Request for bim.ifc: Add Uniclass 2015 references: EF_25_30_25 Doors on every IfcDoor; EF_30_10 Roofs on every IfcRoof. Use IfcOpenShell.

First a look at what the model holds.

```python
import ifcopenshell

model = ifcopenshell.open("bim.ifc")
print(model.schema)
print("classifications:", [c.Name for c in model.by_type("IfcClassification")])
for ifc_class in ("IfcDoor", "IfcRoof", "IfcStair", "IfcWall", "IfcWindow"):
    print(ifc_class, len(model.by_type(ifc_class)))
```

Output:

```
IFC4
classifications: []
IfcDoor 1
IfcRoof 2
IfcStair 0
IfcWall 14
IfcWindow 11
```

```python
import ifcopenshell
import ifcopenshell.api.classification

model = ifcopenshell.open("bim.ifc")

system = ifcopenshell.api.classification.add_classification(model, classification="Uniclass 2015")

codes = {
    "IfcDoor": ("EF_25_30_25", "Doors"),
    "IfcRoof": ("EF_30_10", "Roofs"),
}
for ifc_class, (code, name) in codes.items():
    products = model.by_type(ifc_class)
    ifcopenshell.api.classification.add_reference(
        model, products=products, classification=system, identification=code, name=name
    )
    print(code, len(products))

model.write("bim_updated.ifc")
```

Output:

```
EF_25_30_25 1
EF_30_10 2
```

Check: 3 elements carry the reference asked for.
